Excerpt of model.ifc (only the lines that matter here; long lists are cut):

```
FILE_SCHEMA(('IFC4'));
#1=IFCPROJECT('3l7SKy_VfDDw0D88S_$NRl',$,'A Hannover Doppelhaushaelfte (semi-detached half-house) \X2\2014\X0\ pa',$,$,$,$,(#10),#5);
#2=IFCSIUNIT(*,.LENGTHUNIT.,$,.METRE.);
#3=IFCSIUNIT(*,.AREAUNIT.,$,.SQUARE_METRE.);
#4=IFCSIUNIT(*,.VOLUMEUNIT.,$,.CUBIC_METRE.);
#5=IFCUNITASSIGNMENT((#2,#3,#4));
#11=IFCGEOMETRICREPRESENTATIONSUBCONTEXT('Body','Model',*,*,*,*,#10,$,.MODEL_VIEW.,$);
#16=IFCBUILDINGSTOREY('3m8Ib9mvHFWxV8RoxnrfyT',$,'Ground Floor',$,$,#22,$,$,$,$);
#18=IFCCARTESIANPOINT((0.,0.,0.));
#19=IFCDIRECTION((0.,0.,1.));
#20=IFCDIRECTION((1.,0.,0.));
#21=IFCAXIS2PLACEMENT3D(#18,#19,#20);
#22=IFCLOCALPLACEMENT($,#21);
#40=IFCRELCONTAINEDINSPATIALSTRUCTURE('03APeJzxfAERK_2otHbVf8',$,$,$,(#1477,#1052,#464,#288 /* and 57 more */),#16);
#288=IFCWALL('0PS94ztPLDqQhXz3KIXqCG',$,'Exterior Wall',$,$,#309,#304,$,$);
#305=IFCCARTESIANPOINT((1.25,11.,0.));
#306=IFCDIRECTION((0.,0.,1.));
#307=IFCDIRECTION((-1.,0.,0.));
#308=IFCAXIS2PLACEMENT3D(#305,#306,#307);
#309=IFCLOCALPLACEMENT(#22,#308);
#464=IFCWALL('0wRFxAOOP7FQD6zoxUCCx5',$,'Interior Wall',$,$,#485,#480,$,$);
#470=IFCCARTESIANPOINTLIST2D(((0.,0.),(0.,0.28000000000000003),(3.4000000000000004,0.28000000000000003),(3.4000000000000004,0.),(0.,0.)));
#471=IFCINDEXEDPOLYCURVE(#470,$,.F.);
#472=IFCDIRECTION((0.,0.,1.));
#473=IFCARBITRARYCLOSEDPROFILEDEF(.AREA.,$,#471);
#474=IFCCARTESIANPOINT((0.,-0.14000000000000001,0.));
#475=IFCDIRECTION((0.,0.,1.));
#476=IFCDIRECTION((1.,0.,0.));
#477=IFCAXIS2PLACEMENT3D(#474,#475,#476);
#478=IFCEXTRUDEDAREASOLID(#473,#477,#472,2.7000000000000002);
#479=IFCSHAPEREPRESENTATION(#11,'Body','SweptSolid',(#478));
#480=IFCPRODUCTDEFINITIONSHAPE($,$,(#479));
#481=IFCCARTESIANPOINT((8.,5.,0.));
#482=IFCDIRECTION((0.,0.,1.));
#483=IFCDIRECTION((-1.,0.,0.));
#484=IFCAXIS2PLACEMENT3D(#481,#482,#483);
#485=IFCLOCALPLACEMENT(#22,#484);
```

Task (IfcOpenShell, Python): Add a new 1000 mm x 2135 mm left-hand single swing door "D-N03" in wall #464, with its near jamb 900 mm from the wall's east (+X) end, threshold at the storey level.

```python
import numpy as np
import ifcopenshell
import ifcopenshell.api.feature
import ifcopenshell.api.geometry
import ifcopenshell.api.root
import ifcopenshell.api.spatial
import ifcopenshell.geom
import ifcopenshell.util.element
import ifcopenshell.util.placement
import ifcopenshell.util.representation
import ifcopenshell.util.shape
import ifcopenshell.util.unit

model = ifcopenshell.open("model.ifc")
unit_scale = ifcopenshell.util.unit.calculate_unit_scale(model)
settings = ifcopenshell.geom.settings()


def volume(element):
    """Net volume in cubic metres, openings subtracted."""
    shape = ifcopenshell.geom.create_shape(settings, element)
    return ifcopenshell.util.shape.get_volume(shape.geometry)


wall = model.by_id(464)
storey = ifcopenshell.util.element.get_container(wall, ifc_class="IfcBuildingStorey")
context = ifcopenshell.util.representation.get_context(model, "Model", "Body", "MODEL_VIEW")
before = volume(wall)

width, height, from_end, sill = 1, 2.135, 0.9, 0.0  # metres

# The wall runs along its own X axis, and the end named is its -X end.
wall_shape = ifcopenshell.geom.create_shape(settings, wall)
x, y, z = ifcopenshell.util.shape.get_vertices(wall_shape.geometry).T
start = x.min() + from_end
face, thickness = float(y.min()), float(y.max() - y.min())
wall_matrix = ifcopenshell.util.placement.get_local_placement(wall.ObjectPlacement)
level = ifcopenshell.util.placement.get_local_placement(storey.ObjectPlacement)[2, 3]


def in_wall(x, y):
    """Placement at x, y metres in the wall's axes, at sill height."""
    matrix = wall_matrix.copy()
    matrix[:, 3] = wall_matrix @ np.array([x / unit_scale, y / unit_scale, 0.0, 1.0])
    matrix[2, 3] = level + sill / unit_scale
    return matrix


# Opening: a box that overshoots both wall faces by 50 mm.
opening = ifcopenshell.api.root.create_entity(model, ifc_class="IfcOpeningElement", predefined_type="OPENING")
box = ifcopenshell.api.geometry.add_wall_representation(
    model, context=context, length=width, height=height, thickness=thickness + 0.1
)
ifcopenshell.api.geometry.assign_representation(model, product=opening, representation=box)
ifcopenshell.api.geometry.edit_object_placement(model, product=opening, matrix=in_wall(start, face - 0.05), is_si=False)
ifcopenshell.api.feature.add_feature(model, feature=opening, element=wall)

door = ifcopenshell.api.root.create_entity(model, ifc_class="IfcDoor", name="D-N03", predefined_type="DOOR")
door.OverallWidth, door.OverallHeight = width / unit_scale, height / unit_scale
door.OperationType = "SINGLE_SWING_LEFT"
body = ifcopenshell.api.geometry.add_door_representation(
    model,
    context=context,
    overall_width=door.OverallWidth,
    overall_height=door.OverallHeight,
    operation_type="SINGLE_SWING_LEFT",
    lining_properties={"LiningDepth": thickness / unit_scale, "ThresholdDepth": thickness / unit_scale},
)
ifcopenshell.api.geometry.assign_representation(model, product=door, representation=body)
ifcopenshell.api.spatial.assign_container(model, products=[door], relating_structure=storey)
ifcopenshell.api.feature.add_filling(model, opening=opening, element=door)

# The lining spans the wall, so the door starts at the wall face.
ifcopenshell.api.geometry.edit_object_placement(model, product=door, matrix=in_wall(start, face), is_si=False)

after = volume(wall)

print(f"wall volume {before:.3f} -> {after:.3f} m3")

model.write("model_edited.ifc")
```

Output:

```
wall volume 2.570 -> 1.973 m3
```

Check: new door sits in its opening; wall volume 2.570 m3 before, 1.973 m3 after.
